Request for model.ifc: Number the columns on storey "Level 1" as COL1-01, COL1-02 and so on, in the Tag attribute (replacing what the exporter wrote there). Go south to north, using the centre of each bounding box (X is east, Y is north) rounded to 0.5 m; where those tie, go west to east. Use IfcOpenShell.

First a look at what the model holds.

```python
import ifcopenshell
import ifcopenshell.util.element
import ifcopenshell.util.placement

model = ifcopenshell.open("model.ifc")
print(model.schema)
storey = next(s for s in model.by_type("IfcBuildingStorey") if s.Name == "Level 1")
columns = [e for e in ifcopenshell.util.element.get_decomposition(storey) if e.is_a("IfcColumn")]
for e in sorted(columns, key=lambda e: e.id()):
    origin = ifcopenshell.util.placement.get_local_placement(e.ObjectPlacement)[:3, 3]
    print(e.id(), e.Tag, e.Name, origin.round(2) + 0.0, sep=" | ")
```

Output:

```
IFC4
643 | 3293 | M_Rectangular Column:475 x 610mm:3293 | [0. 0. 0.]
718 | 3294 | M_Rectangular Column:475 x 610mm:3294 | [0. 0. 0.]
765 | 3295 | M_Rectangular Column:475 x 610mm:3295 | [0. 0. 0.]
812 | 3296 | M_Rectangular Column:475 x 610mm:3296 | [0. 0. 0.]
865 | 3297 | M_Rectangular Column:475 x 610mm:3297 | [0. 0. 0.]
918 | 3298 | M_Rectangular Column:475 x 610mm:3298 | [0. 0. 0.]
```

```python
import ifcopenshell
import ifcopenshell.geom
import ifcopenshell.util.element
import ifcopenshell.util.shape

model = ifcopenshell.open("model.ifc")
settings = ifcopenshell.geom.settings()
settings.set("use-world-coords", True)


def centre(element):
    shape = ifcopenshell.geom.create_shape(settings, element)
    return ifcopenshell.util.shape.get_bbox_centroid(shape.geometry)


storey = next(s for s in model.by_type("IfcBuildingStorey") if s.Name == "Level 1")
columns = [e for e in ifcopenshell.util.element.get_decomposition(storey) if e.is_a("IfcColumn")]

# Insertion points can sit at a corner or the storey origin, so sort by the geometry (in metres).
centres = {e: centre(e) for e in columns}
columns.sort(key=lambda e: (round(centres[e][1] / 0.5), centres[e][0]))

for i, e in enumerate(columns, start=1):
    number = f"COL1-{i:02d}"
    e.Tag = number
    print(e.id(), number)

model.write("model-out.ifc")
```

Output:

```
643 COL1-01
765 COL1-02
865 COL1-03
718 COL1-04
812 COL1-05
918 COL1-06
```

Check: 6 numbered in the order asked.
